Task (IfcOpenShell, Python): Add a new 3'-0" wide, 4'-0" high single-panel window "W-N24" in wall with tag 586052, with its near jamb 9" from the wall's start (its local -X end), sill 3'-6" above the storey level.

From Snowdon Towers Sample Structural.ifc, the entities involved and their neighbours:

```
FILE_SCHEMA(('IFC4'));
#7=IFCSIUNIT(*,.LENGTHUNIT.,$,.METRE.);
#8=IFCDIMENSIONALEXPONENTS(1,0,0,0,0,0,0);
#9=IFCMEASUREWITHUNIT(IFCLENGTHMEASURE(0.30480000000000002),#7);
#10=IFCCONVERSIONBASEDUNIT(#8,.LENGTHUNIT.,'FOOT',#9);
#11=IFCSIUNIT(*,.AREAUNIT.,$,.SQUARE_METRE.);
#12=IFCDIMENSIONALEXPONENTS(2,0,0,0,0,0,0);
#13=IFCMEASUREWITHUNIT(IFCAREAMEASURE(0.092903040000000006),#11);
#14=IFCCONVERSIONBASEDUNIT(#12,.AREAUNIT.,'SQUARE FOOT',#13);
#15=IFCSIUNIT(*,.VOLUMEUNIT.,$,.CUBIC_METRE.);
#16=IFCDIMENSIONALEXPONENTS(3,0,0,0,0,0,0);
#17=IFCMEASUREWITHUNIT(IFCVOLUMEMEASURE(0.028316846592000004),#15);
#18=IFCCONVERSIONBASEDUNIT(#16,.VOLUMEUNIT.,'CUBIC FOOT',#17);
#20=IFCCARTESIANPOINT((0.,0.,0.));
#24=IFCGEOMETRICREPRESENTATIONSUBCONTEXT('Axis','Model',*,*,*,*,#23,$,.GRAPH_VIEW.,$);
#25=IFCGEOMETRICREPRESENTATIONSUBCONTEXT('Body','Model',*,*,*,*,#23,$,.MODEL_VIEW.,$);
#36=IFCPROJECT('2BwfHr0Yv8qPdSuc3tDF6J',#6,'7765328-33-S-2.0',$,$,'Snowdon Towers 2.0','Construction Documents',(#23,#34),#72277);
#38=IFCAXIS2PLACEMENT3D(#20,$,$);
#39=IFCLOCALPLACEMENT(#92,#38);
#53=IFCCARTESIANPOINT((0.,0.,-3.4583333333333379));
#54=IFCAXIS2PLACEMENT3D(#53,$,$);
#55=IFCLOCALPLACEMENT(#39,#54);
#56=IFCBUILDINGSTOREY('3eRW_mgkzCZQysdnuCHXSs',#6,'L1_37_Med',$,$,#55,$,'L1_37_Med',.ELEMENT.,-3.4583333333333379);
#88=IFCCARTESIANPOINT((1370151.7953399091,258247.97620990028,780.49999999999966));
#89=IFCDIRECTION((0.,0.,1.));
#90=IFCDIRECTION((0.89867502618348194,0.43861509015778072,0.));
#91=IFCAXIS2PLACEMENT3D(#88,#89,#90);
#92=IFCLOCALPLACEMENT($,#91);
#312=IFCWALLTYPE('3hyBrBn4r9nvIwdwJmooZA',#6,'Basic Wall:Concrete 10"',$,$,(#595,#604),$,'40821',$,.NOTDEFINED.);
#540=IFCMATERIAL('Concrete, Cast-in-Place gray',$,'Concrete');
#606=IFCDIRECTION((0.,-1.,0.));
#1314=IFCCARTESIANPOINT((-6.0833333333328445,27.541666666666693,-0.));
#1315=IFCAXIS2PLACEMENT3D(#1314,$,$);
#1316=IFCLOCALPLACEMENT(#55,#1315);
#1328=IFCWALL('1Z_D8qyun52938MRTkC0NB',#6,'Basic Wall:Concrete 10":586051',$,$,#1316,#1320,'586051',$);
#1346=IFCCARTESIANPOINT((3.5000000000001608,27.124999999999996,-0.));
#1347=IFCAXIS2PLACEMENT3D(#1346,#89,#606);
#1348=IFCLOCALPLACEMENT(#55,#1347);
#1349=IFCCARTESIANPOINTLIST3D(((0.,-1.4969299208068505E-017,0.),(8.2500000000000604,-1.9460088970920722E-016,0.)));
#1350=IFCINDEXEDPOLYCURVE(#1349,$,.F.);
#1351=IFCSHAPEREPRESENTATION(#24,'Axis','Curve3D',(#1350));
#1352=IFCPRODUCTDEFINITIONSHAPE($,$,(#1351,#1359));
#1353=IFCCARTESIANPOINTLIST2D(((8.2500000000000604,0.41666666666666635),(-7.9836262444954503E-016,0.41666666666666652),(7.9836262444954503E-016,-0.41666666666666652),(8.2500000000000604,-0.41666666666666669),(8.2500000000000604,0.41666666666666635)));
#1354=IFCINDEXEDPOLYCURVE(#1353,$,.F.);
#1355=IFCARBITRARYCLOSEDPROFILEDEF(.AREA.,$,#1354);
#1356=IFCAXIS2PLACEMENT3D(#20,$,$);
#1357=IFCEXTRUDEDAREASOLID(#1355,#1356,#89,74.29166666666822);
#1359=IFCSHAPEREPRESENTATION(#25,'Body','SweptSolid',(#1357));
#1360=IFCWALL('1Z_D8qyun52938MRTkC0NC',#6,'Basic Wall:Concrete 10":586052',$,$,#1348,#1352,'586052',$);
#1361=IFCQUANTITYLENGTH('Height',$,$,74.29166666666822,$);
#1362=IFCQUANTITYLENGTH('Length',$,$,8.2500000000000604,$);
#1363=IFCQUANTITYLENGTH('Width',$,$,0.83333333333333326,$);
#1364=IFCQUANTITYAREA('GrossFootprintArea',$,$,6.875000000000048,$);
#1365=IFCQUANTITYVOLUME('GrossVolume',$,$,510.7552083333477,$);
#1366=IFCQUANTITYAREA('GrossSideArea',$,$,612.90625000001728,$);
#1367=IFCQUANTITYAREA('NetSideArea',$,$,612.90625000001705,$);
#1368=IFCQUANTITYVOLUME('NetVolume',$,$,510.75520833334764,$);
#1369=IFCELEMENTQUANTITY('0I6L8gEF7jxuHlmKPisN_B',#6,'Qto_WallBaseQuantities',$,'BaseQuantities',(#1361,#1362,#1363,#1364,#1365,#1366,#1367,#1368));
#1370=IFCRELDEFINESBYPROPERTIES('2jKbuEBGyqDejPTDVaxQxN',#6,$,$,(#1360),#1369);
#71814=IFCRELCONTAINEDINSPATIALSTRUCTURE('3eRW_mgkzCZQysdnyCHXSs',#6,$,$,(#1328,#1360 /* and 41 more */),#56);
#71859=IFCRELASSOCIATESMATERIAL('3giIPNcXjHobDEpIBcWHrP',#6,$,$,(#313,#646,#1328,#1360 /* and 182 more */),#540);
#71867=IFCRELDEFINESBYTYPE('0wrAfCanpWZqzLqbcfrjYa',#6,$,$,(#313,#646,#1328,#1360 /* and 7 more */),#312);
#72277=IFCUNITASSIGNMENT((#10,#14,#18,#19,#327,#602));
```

```python
import numpy as np
import ifcopenshell
import ifcopenshell.api.feature
import ifcopenshell.api.geometry
import ifcopenshell.api.pset
import ifcopenshell.api.root
import ifcopenshell.api.spatial
import ifcopenshell.geom
import ifcopenshell.util.element
import ifcopenshell.util.placement
import ifcopenshell.util.representation
import ifcopenshell.util.shape
import ifcopenshell.util.unit

model = ifcopenshell.open("Snowdon Towers Sample Structural.ifc")
unit_scale = ifcopenshell.util.unit.calculate_unit_scale(model)
area_scale = ifcopenshell.util.unit.calculate_unit_scale(model, "AREAUNIT")
volume_scale = ifcopenshell.util.unit.calculate_unit_scale(model, "VOLUMEUNIT")
settings = ifcopenshell.geom.settings()


def volume(element):
    """Net volume in cubic metres, openings subtracted."""
    shape = ifcopenshell.geom.create_shape(settings, element)
    return ifcopenshell.util.shape.get_volume(shape.geometry)


wall = model.by_guid("1Z_D8qyun52938MRTkC0NC")
storey = ifcopenshell.util.element.get_container(wall, ifc_class="IfcBuildingStorey")
context = ifcopenshell.util.representation.get_context(model, "Model", "Body", "MODEL_VIEW")
before = volume(wall)

width, height, from_end, sill = 0.9144, 1.2192, 0.2286, 1.0668  # metres

# The wall runs along its own X axis, and the end named is its -X end.
wall_shape = ifcopenshell.geom.create_shape(settings, wall)
x, y, z = ifcopenshell.util.shape.get_vertices(wall_shape.geometry).T
start = x.min() + from_end
face, thickness = float(y.min()), float(y.max() - y.min())
wall_matrix = ifcopenshell.util.placement.get_local_placement(wall.ObjectPlacement)
level = ifcopenshell.util.placement.get_local_placement(storey.ObjectPlacement)[2, 3]


def in_wall(x, y):
    """Placement at x, y metres in the wall's axes, at sill height."""
    matrix = wall_matrix.copy()
    matrix[:, 3] = wall_matrix @ np.array([x / unit_scale, y / unit_scale, 0.0, 1.0])
    matrix[2, 3] = level + sill / unit_scale
    return matrix


# Opening: a box that overshoots both wall faces by 50 mm.
opening = ifcopenshell.api.root.create_entity(model, ifc_class="IfcOpeningElement", predefined_type="OPENING")
box = ifcopenshell.api.geometry.add_wall_representation(
    model, context=context, length=width, height=height, thickness=thickness + 0.1
)
ifcopenshell.api.geometry.assign_representation(model, product=opening, representation=box)
ifcopenshell.api.geometry.edit_object_placement(model, product=opening, matrix=in_wall(start, face - 0.05), is_si=False)
ifcopenshell.api.feature.add_feature(model, feature=opening, element=wall)

window = ifcopenshell.api.root.create_entity(model, ifc_class="IfcWindow", name="W-N24", predefined_type="WINDOW")
window.OverallWidth, window.OverallHeight = width / unit_scale, height / unit_scale
window.PartitioningType = "SINGLE_PANEL"
body = ifcopenshell.api.geometry.add_window_representation(
    model,
    context=context,
    overall_width=window.OverallWidth,
    overall_height=window.OverallHeight,
    partition_type="SINGLE_PANEL",
)
ifcopenshell.api.geometry.assign_representation(model, product=window, representation=body)
ifcopenshell.api.spatial.assign_container(model, products=[window], relating_structure=storey)
ifcopenshell.api.feature.add_filling(model, opening=opening, element=window)

# Centre the window in the wall's thickness.
ifcopenshell.api.geometry.edit_object_placement(model, product=window, matrix=in_wall(start, face), is_si=False)
window_shape = ifcopenshell.geom.create_shape(settings, window)
depth = ifcopenshell.util.shape.get_vertices(window_shape.geometry)[:, 1]
offset = face + thickness / 2 - (depth.min() + depth.max()) / 2
ifcopenshell.api.geometry.edit_object_placement(model, product=window, matrix=in_wall(start, offset), is_si=False)

after = volume(wall)

# Update the wall's stored quantities.
qto = model.by_id(ifcopenshell.util.element.get_pset(wall, "Qto_WallBaseQuantities", should_inherit=False)["id"])
ifcopenshell.api.pset.edit_qto(model, qto=qto, properties={
    "NetSideArea": after / thickness / area_scale,
    "NetVolume": after / volume_scale,
})

print(f"wall volume {before:.3f} -> {after:.3f} m3")

model.write("Snowdon Towers Sample Structural-out.ifc")
```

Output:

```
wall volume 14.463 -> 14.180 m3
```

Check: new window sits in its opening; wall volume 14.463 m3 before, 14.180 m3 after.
